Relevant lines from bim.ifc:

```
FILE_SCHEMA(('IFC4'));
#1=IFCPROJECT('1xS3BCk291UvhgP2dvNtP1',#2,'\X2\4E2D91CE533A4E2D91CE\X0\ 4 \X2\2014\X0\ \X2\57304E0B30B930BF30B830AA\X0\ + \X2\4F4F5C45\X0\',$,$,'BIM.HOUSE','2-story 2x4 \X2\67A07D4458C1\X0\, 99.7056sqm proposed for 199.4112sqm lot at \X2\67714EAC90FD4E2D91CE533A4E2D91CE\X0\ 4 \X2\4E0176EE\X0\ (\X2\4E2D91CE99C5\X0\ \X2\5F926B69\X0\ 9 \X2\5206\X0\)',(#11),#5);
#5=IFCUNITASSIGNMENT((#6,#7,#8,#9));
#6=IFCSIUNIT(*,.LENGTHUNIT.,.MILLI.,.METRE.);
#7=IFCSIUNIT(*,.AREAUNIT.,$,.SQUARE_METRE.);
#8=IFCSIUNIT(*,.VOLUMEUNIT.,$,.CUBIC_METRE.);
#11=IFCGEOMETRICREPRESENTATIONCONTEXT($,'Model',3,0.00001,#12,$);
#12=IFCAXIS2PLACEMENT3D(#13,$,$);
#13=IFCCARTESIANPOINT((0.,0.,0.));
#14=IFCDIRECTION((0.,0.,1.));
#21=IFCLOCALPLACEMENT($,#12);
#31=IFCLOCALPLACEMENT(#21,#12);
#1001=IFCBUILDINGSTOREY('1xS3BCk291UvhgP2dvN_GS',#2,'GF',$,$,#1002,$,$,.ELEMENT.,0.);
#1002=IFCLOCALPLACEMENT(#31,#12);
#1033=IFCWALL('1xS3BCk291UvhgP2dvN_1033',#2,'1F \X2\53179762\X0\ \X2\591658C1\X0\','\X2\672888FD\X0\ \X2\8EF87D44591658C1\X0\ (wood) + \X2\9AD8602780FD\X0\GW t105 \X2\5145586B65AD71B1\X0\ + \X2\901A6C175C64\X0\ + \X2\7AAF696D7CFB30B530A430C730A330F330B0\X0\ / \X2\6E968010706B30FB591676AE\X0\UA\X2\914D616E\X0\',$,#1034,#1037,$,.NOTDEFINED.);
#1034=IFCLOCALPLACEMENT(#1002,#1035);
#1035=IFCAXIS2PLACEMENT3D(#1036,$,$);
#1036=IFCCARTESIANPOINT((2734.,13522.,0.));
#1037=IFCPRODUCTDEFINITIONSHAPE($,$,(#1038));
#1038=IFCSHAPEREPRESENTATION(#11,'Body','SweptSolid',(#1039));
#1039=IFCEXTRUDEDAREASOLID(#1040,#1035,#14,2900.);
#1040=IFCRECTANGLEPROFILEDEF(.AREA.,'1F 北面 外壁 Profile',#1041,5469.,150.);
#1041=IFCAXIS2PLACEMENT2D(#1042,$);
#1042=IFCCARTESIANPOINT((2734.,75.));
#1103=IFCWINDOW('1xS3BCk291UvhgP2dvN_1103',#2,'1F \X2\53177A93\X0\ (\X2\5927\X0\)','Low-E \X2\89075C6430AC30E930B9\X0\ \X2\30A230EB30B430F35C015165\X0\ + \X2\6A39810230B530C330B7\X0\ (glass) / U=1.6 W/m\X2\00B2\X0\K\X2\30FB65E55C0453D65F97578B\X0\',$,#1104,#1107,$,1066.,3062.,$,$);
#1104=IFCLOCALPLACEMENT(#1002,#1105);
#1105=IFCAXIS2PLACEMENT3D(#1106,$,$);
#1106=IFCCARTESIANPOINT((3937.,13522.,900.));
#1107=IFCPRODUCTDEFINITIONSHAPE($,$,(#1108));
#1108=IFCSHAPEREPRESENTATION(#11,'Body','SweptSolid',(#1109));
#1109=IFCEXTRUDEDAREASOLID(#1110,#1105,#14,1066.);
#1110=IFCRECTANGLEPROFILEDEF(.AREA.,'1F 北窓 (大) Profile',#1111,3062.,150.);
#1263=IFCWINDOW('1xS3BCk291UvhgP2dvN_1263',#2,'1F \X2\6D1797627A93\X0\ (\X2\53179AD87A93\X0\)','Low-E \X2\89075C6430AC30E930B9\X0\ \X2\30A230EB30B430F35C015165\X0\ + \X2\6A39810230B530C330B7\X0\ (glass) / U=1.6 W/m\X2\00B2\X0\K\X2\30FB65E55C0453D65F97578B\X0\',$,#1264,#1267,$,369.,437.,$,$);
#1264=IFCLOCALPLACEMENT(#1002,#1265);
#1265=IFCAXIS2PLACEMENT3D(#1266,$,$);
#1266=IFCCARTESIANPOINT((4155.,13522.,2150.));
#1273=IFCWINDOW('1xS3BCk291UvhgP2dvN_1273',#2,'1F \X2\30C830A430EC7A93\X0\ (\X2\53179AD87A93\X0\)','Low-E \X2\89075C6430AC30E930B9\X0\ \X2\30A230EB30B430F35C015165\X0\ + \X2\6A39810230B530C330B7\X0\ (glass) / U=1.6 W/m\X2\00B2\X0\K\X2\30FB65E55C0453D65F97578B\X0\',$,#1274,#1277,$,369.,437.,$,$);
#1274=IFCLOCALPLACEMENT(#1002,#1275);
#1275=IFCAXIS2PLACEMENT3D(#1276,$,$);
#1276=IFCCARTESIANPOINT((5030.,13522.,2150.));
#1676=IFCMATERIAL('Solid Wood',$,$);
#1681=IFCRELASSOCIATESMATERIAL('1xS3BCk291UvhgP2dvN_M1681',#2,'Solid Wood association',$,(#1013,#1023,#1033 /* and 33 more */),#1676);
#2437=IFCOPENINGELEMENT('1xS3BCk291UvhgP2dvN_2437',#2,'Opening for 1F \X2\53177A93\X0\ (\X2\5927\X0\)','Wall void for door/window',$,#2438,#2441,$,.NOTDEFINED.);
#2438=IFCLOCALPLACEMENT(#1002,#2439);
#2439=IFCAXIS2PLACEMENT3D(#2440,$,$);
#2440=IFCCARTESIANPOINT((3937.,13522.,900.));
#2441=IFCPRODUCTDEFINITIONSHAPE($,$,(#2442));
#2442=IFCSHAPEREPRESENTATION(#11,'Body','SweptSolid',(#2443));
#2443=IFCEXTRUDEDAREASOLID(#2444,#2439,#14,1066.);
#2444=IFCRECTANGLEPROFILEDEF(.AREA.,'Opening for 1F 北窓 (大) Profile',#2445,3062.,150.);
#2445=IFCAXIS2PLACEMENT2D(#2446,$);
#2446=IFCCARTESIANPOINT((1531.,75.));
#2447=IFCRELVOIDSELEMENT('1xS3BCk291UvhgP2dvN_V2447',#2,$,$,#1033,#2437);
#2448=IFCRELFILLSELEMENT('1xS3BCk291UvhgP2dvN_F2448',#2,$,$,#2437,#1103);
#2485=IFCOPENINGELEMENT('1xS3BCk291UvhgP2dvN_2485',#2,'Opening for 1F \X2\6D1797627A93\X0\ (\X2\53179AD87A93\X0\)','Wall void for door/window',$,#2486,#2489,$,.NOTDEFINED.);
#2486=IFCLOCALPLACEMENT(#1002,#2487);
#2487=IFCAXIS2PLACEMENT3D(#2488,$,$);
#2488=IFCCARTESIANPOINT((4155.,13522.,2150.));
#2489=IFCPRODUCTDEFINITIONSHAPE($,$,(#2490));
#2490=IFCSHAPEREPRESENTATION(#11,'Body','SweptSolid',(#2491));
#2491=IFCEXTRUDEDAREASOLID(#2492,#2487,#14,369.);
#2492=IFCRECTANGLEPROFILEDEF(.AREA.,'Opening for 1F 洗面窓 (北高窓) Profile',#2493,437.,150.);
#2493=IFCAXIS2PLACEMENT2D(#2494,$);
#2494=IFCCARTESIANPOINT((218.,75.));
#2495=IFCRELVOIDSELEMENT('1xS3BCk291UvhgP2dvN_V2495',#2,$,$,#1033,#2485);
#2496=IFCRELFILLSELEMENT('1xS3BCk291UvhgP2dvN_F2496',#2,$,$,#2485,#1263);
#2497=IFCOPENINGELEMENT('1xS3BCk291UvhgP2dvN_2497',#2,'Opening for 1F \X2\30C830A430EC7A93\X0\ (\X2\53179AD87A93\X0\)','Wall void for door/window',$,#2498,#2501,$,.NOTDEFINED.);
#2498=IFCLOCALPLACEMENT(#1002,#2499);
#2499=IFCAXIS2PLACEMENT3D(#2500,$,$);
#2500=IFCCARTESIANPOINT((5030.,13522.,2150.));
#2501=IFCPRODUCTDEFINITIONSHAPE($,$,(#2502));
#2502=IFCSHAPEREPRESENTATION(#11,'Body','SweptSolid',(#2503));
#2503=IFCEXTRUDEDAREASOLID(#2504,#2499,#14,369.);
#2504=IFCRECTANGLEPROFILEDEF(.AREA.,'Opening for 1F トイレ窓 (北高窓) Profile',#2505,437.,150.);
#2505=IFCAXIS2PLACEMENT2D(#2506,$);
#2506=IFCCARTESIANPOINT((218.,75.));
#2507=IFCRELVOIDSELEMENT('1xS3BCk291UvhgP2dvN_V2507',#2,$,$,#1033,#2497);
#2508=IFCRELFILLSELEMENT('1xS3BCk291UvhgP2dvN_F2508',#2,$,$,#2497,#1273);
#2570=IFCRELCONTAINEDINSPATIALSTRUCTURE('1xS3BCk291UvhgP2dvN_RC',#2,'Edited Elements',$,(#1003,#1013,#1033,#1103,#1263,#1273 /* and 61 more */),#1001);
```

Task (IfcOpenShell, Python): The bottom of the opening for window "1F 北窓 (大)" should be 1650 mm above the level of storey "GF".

```python
import numpy as np
import ifcopenshell
import ifcopenshell.api.geometry
import ifcopenshell.geom
import ifcopenshell.util.element
import ifcopenshell.util.placement
import ifcopenshell.util.shape
import ifcopenshell.util.unit

model = ifcopenshell.open("bim.ifc")
unit_scale = ifcopenshell.util.unit.calculate_unit_scale(model)

window = model.by_guid("1xS3BCk291UvhgP2dvN_1103")
opening = window.FillsVoids[0].RelatingOpeningElement
storey = ifcopenshell.util.element.get_container(window, ifc_class="IfcBuildingStorey")
level = ifcopenshell.util.placement.get_local_placement(storey.ObjectPlacement)[2, 3]

# The opening's origin need not be at the sill, so measure its lowest point.
shape = ifcopenshell.geom.create_shape(ifcopenshell.geom.settings(), opening)
bottom = ifcopenshell.util.shape.get_shape_bottom_elevation(shape, shape.geometry) / unit_scale
dz = level + 1.65 / unit_scale - bottom

shift = np.array([0.0, 0.0, dz])
# The window is not placed relative to its opening, so move both.
for product in (opening, window):
    matrix = ifcopenshell.util.placement.get_local_placement(product.ObjectPlacement)
    matrix[:3, 3] += shift
    ifcopenshell.api.geometry.edit_object_placement(model, product=product, matrix=matrix, is_si=False)

print(f"moved by {dz * unit_scale:+.3f} m")

model.write("bim_updated.ifc")
```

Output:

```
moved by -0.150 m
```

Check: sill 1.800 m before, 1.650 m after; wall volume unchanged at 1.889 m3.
